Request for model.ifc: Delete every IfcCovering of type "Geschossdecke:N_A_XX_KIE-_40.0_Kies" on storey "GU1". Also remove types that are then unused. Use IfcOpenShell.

First a look at what the model holds.

```python
import ifcopenshell
import ifcopenshell.util.element

model = ifcopenshell.open("model.ifc")
print(model.schema)
storey = next(s for s in model.by_type("IfcBuildingStorey") if s.Name == "GU1")
coverings = [e for e in ifcopenshell.util.element.get_decomposition(storey) if e.is_a("IfcCovering")]
seen = {}
for e in coverings:
    element_type = ifcopenshell.util.element.get_type(e)
    name = element_type.Name if element_type not in (None, e) else None
    seen[name] = seen.get(name, 0) + 1
for name, count in sorted(seen.items(), key=str):
    print(count, "x", name)
```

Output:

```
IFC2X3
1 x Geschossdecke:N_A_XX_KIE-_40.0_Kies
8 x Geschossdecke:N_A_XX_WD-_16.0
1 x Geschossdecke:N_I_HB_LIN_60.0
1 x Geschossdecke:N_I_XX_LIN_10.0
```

```python
import ifcopenshell
import ifcopenshell.api.root
import ifcopenshell.util.element

model = ifcopenshell.open("model.ifc")

storey = next(s for s in model.by_type("IfcBuildingStorey") if s.Name == "GU1")
coverings = [e for e in ifcopenshell.util.element.get_decomposition(storey) if e.is_a("IfcCovering")]
targets = [e for e in coverings if (t := ifcopenshell.util.element.get_type(e)) not in (None, e) and t.Name == "Geschossdecke:N_A_XX_KIE-_40.0_Kies"]
types = {ifcopenshell.util.element.get_type(e) for e in targets} - {None, *targets}

for e in targets:
    ifcopenshell.api.root.remove_product(model, product=e)
print(len(targets), "removed")

unused = [t for t in types if not ifcopenshell.util.element.get_types(t)]
for t in unused:
    ifcopenshell.api.root.remove_product(model, product=t)
print(len(unused), "unused types removed")

model.write("model_rev.ifc")
```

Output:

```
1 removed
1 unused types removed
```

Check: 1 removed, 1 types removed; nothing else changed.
